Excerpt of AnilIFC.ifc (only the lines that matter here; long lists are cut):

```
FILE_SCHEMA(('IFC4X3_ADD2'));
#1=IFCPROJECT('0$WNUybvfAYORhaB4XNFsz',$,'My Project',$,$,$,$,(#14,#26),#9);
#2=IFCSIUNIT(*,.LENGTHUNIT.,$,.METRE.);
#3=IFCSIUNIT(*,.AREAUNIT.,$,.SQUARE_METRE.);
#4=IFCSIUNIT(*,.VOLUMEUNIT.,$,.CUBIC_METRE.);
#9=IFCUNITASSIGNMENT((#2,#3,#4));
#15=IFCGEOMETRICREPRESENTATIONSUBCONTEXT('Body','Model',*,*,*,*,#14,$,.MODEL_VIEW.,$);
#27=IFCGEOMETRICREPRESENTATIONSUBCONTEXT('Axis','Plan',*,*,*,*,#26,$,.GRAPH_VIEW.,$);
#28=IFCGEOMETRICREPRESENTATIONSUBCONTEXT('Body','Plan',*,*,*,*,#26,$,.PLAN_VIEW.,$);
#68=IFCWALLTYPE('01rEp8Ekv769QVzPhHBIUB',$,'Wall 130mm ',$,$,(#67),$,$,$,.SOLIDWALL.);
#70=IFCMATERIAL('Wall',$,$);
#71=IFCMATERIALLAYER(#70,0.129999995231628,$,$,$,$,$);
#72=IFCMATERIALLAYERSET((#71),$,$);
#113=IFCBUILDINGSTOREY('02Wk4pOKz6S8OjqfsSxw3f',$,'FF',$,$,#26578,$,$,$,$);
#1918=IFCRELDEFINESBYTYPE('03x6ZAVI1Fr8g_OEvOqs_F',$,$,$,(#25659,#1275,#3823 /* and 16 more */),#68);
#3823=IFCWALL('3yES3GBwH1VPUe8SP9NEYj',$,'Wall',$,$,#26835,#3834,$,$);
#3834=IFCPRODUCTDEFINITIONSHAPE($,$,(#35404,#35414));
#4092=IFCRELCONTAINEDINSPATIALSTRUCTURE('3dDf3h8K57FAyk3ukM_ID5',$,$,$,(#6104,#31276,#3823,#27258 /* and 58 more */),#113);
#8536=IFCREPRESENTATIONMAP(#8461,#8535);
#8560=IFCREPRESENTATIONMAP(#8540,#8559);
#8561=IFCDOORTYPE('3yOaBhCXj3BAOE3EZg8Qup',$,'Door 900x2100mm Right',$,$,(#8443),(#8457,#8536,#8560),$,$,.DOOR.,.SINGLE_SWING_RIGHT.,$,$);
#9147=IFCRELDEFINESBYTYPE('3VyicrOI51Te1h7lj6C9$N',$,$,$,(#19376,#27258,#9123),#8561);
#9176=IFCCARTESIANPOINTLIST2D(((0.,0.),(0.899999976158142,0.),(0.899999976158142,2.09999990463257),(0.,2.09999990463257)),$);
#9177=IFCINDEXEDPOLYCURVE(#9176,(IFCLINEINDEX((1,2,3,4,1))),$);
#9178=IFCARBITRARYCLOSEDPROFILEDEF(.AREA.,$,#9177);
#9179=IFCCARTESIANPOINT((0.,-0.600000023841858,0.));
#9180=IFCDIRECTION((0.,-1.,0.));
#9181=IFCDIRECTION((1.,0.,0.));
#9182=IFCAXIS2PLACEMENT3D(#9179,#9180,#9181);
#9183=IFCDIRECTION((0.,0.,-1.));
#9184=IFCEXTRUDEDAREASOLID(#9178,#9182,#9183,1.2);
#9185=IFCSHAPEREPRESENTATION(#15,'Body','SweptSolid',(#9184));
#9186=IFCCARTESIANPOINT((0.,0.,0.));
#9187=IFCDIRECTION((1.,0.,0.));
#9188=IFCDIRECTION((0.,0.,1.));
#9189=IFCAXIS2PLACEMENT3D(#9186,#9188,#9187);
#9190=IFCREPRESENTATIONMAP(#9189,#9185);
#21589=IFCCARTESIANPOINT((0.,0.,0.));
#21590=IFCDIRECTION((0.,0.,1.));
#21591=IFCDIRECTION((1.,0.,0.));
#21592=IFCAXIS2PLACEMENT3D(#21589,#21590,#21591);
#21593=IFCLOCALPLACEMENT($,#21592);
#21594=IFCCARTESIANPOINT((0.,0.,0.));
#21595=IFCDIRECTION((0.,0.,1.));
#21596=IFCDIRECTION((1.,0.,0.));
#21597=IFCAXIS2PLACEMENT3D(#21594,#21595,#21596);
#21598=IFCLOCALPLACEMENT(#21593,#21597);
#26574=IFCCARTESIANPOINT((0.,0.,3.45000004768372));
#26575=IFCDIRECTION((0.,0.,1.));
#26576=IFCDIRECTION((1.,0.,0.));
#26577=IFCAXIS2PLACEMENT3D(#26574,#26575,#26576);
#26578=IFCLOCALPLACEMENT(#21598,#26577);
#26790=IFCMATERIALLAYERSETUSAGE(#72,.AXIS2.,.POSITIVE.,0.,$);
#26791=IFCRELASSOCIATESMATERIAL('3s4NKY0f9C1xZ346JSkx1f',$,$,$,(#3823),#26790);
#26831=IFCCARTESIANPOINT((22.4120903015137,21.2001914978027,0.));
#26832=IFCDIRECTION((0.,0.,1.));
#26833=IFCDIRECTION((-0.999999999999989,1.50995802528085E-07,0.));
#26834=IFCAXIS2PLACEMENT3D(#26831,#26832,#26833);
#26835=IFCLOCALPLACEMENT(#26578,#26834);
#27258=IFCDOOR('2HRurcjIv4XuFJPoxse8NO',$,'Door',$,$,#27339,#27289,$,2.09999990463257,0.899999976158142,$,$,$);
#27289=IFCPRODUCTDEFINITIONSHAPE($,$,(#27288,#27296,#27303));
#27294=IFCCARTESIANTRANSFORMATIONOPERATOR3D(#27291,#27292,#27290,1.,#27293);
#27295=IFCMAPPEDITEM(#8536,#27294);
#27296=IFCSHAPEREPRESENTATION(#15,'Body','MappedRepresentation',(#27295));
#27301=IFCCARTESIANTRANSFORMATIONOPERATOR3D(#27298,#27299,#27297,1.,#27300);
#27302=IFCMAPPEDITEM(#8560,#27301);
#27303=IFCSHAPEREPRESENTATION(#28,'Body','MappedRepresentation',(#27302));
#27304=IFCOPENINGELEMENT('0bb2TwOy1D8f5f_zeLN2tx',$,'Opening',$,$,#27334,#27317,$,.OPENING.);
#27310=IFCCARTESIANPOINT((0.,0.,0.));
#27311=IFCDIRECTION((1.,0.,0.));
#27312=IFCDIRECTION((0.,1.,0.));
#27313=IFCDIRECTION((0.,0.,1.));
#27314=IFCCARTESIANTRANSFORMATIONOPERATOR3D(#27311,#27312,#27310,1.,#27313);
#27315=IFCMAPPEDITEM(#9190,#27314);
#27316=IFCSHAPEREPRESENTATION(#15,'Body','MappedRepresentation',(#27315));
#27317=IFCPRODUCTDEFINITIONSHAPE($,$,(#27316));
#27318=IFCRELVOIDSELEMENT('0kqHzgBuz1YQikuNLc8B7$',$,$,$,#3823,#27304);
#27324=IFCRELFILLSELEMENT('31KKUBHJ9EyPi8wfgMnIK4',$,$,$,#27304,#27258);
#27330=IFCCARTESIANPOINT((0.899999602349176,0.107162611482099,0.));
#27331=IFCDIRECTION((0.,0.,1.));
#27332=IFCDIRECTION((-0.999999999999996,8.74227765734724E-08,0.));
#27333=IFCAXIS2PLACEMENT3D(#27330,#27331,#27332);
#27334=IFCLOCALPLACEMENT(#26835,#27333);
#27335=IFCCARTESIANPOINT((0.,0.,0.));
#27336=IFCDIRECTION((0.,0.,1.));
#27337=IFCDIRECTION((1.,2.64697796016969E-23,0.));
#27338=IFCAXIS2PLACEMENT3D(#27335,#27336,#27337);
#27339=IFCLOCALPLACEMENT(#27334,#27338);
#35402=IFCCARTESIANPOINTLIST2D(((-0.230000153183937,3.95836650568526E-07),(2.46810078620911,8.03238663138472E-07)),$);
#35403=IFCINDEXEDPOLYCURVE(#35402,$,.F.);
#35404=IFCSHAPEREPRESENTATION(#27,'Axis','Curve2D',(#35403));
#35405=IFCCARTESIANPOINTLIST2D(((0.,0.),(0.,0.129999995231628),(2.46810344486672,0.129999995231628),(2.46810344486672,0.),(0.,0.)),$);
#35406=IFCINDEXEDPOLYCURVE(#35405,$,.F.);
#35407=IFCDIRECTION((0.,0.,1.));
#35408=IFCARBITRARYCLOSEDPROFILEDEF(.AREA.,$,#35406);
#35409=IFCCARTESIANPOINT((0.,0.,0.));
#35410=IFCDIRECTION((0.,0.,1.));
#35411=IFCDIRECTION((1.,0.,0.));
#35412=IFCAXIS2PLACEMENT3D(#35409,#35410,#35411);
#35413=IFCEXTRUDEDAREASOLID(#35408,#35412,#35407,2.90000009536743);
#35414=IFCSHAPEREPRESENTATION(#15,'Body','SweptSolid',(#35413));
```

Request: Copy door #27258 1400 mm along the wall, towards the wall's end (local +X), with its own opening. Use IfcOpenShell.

```python
import ifcopenshell
import ifcopenshell.api.feature
import ifcopenshell.api.geometry
import ifcopenshell.api.root
import ifcopenshell.geom
import ifcopenshell.util.element
import ifcopenshell.util.placement
import ifcopenshell.util.shape
import ifcopenshell.util.unit

model = ifcopenshell.open("AnilIFC.ifc")
unit_scale = ifcopenshell.util.unit.calculate_unit_scale(model)
settings = ifcopenshell.geom.settings()


def volume(element):
    """Net volume in cubic metres, openings subtracted."""
    shape = ifcopenshell.geom.create_shape(settings, element)
    return ifcopenshell.util.shape.get_volume(shape.geometry)


door = model.by_id(27258)
opening = door.FillsVoids[0].RelatingOpeningElement
wall = opening.VoidsElements[0].RelatingBuildingElement
before = volume(wall)
shift = ifcopenshell.util.placement.get_local_placement(wall.ObjectPlacement)[:3, 0] * 1.4 / unit_scale

# copy_class copies the void relationship, type, container and properties, but no geometry.
new_opening = ifcopenshell.api.root.copy_class(model, product=opening)
new_opening.Representation = ifcopenshell.util.element.copy_deep(
    model, opening.Representation, exclude=["IfcGeometricRepresentationContext", "IfcRepresentationMap"]
)
new_door = ifcopenshell.api.root.copy_class(model, product=door)
new_door.Representation = ifcopenshell.util.element.copy_deep(
    model, door.Representation, exclude=["IfcGeometricRepresentationContext", "IfcRepresentationMap"]
)
ifcopenshell.api.feature.add_filling(model, opening=new_opening, element=new_door)

for old, new in ((opening, new_opening), (door, new_door)):
    matrix = ifcopenshell.util.placement.get_local_placement(old.ObjectPlacement)
    matrix[:3, 3] += shift
    ifcopenshell.api.geometry.edit_object_placement(model, product=new, matrix=matrix, is_si=False)

after = volume(wall)

print(f"wall volume {before:.3f} -> {after:.3f} m3")

model.write("AnilIFC-out.ifc")
```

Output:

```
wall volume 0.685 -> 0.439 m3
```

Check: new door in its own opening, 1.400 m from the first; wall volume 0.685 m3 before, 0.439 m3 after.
